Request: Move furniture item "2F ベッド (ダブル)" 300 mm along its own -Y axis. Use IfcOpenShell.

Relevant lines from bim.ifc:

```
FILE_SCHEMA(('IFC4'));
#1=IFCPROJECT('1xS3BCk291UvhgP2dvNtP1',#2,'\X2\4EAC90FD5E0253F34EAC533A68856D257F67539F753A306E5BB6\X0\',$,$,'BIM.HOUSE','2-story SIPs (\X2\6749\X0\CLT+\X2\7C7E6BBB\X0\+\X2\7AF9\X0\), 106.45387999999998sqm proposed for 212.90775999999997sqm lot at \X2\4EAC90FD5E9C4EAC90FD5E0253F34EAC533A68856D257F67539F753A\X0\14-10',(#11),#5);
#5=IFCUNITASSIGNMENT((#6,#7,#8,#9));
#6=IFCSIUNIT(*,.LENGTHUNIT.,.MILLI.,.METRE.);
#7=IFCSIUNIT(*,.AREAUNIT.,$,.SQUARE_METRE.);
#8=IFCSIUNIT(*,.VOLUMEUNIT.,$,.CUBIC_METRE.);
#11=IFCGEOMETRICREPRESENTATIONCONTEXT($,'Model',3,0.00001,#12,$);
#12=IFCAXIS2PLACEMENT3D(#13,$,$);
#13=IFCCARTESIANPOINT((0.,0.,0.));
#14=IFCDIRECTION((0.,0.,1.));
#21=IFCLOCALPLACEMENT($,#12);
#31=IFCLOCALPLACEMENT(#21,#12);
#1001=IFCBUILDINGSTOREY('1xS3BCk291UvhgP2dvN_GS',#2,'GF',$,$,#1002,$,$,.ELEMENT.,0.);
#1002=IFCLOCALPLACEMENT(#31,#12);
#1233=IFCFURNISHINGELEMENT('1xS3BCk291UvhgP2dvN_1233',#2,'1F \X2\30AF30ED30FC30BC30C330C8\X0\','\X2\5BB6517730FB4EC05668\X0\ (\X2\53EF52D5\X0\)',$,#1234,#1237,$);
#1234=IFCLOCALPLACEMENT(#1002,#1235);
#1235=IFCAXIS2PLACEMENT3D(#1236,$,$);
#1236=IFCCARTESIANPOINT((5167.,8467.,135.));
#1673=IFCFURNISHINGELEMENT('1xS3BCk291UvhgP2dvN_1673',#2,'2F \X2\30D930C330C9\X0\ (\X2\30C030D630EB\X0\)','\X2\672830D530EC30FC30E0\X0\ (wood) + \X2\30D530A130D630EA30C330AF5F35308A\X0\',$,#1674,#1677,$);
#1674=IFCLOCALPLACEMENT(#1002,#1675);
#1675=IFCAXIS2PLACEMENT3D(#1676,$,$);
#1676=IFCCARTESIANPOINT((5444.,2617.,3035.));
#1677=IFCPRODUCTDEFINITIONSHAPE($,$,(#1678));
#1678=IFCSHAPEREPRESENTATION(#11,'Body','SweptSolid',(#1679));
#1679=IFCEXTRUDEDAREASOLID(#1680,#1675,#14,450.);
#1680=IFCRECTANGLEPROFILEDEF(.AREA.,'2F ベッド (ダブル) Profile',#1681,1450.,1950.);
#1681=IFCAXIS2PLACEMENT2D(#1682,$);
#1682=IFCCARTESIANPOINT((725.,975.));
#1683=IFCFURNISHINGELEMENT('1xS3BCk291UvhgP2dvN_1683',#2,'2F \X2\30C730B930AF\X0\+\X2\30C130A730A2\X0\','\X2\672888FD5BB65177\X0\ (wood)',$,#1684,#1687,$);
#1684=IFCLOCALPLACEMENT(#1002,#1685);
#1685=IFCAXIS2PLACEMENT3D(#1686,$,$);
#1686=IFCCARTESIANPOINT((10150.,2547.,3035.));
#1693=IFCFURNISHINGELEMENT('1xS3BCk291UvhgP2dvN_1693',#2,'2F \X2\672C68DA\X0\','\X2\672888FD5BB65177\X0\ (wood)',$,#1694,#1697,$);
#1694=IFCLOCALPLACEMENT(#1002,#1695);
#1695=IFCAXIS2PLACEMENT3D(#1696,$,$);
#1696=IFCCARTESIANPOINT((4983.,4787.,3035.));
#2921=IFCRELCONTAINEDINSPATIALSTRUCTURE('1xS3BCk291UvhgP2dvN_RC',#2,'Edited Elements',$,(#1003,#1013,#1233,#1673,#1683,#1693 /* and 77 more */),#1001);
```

```python
import ifcopenshell
import ifcopenshell.api.geometry
import ifcopenshell.util.placement

model = ifcopenshell.open("bim.ifc")

item = model.by_guid("1xS3BCk291UvhgP2dvN_1673")
matrix = ifcopenshell.util.placement.get_local_placement(item.ObjectPlacement)
matrix[:3, 3] -= matrix[:3, 1] * 300.0
ifcopenshell.api.geometry.edit_object_placement(model, product=item, matrix=matrix, is_si=False)

print(ifcopenshell.util.placement.get_local_placement(item.ObjectPlacement).round(3) + 0.0)

model.write("bim_v2.ifc")
```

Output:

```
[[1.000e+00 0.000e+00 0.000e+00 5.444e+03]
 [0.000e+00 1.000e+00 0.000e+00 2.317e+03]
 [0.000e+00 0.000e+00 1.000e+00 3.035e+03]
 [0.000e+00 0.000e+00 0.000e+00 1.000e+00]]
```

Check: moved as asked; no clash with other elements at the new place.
